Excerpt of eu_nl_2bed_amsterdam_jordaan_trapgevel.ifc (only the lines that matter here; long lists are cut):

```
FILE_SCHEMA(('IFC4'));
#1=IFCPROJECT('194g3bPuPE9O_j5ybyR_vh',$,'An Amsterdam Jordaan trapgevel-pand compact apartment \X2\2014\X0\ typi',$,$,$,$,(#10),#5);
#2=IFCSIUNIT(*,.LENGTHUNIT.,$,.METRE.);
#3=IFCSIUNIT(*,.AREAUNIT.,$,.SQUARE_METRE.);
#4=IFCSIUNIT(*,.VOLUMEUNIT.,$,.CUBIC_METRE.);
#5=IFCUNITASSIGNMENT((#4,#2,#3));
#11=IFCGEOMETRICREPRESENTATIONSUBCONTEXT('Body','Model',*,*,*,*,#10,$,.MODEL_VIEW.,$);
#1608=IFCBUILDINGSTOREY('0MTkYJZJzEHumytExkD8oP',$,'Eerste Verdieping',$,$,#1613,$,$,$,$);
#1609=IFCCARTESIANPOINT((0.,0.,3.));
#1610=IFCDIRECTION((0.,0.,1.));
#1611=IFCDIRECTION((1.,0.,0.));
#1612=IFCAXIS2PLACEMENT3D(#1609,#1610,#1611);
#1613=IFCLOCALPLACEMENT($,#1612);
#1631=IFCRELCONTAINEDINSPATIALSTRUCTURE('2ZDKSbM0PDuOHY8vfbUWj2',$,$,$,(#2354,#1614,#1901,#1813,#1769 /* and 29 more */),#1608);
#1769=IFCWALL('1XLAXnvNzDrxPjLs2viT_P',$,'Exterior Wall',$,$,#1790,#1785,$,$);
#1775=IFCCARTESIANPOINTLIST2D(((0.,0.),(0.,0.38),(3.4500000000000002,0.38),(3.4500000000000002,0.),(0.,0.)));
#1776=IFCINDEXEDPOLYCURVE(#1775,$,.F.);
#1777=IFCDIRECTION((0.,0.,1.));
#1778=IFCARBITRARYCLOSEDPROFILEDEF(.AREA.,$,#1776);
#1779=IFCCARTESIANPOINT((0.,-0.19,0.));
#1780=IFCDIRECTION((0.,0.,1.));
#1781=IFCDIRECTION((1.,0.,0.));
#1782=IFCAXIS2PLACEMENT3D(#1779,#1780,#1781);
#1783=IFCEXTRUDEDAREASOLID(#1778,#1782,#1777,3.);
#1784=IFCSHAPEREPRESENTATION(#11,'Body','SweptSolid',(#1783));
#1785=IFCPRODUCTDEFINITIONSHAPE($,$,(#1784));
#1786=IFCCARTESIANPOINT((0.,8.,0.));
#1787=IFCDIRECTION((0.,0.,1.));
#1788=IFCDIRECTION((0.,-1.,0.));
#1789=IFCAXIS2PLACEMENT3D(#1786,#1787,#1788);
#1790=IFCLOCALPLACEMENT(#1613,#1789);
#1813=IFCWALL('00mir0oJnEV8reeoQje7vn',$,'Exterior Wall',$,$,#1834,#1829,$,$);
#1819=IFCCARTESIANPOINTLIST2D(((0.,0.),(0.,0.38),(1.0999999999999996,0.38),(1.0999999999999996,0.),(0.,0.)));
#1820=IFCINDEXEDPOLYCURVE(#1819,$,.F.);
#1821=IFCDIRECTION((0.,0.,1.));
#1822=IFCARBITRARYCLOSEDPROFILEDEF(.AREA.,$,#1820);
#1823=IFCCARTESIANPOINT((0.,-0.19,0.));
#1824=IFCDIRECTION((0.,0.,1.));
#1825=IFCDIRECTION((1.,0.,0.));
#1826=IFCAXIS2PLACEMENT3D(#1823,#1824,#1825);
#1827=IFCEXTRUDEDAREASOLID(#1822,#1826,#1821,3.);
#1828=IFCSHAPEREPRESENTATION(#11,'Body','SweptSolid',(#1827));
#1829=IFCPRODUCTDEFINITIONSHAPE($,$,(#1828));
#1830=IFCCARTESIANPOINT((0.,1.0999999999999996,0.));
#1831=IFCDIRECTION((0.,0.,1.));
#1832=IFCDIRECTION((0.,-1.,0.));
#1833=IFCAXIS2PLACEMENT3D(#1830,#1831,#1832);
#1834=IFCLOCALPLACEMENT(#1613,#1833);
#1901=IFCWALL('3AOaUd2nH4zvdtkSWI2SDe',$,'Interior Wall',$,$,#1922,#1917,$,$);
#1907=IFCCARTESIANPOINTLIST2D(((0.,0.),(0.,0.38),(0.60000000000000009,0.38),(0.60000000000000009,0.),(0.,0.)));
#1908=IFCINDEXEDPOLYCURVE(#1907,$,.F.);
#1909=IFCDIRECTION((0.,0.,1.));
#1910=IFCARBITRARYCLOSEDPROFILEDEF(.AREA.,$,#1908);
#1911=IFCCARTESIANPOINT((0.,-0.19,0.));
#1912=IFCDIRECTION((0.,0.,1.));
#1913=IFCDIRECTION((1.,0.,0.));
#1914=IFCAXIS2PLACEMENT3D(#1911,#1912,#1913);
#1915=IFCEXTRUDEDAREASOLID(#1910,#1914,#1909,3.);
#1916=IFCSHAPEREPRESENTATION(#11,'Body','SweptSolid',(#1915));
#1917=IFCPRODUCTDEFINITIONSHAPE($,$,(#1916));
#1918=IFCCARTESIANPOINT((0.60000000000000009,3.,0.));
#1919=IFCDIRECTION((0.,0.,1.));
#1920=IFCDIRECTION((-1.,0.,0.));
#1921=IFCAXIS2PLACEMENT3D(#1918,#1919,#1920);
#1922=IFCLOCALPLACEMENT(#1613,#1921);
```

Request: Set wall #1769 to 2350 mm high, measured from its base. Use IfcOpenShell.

```python
import ifcopenshell
import ifcopenshell.geom
import ifcopenshell.util.representation
import ifcopenshell.util.shape
import ifcopenshell.util.unit

model = ifcopenshell.open("eu_nl_2bed_amsterdam_jordaan_trapgevel.ifc")
unit_scale = ifcopenshell.util.unit.calculate_unit_scale(model)
settings = ifcopenshell.geom.settings()


def volume(element):
    """Net volume in cubic metres, openings subtracted."""
    shape = ifcopenshell.geom.create_shape(settings, element)
    return ifcopenshell.util.shape.get_volume(shape.geometry)


wall = model.by_guid("1XLAXnvNzDrxPjLs2viT_P")
before = volume(wall)

body = ifcopenshell.util.representation.get_representation(wall, "Model", "Body")
solid = body.Items[0]
old_height = solid.Depth
solid.Depth = 2.35 / unit_scale
after = volume(wall)

print(f"height {old_height:g} -> {solid.Depth:g}, volume {before:.3f} -> {after:.3f} m3")

model.write("eu_nl_2bed_amsterdam_jordaan_trapgevel_rev.ifc")
```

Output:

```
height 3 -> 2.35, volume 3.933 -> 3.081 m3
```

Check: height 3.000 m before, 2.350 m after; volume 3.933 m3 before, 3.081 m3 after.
